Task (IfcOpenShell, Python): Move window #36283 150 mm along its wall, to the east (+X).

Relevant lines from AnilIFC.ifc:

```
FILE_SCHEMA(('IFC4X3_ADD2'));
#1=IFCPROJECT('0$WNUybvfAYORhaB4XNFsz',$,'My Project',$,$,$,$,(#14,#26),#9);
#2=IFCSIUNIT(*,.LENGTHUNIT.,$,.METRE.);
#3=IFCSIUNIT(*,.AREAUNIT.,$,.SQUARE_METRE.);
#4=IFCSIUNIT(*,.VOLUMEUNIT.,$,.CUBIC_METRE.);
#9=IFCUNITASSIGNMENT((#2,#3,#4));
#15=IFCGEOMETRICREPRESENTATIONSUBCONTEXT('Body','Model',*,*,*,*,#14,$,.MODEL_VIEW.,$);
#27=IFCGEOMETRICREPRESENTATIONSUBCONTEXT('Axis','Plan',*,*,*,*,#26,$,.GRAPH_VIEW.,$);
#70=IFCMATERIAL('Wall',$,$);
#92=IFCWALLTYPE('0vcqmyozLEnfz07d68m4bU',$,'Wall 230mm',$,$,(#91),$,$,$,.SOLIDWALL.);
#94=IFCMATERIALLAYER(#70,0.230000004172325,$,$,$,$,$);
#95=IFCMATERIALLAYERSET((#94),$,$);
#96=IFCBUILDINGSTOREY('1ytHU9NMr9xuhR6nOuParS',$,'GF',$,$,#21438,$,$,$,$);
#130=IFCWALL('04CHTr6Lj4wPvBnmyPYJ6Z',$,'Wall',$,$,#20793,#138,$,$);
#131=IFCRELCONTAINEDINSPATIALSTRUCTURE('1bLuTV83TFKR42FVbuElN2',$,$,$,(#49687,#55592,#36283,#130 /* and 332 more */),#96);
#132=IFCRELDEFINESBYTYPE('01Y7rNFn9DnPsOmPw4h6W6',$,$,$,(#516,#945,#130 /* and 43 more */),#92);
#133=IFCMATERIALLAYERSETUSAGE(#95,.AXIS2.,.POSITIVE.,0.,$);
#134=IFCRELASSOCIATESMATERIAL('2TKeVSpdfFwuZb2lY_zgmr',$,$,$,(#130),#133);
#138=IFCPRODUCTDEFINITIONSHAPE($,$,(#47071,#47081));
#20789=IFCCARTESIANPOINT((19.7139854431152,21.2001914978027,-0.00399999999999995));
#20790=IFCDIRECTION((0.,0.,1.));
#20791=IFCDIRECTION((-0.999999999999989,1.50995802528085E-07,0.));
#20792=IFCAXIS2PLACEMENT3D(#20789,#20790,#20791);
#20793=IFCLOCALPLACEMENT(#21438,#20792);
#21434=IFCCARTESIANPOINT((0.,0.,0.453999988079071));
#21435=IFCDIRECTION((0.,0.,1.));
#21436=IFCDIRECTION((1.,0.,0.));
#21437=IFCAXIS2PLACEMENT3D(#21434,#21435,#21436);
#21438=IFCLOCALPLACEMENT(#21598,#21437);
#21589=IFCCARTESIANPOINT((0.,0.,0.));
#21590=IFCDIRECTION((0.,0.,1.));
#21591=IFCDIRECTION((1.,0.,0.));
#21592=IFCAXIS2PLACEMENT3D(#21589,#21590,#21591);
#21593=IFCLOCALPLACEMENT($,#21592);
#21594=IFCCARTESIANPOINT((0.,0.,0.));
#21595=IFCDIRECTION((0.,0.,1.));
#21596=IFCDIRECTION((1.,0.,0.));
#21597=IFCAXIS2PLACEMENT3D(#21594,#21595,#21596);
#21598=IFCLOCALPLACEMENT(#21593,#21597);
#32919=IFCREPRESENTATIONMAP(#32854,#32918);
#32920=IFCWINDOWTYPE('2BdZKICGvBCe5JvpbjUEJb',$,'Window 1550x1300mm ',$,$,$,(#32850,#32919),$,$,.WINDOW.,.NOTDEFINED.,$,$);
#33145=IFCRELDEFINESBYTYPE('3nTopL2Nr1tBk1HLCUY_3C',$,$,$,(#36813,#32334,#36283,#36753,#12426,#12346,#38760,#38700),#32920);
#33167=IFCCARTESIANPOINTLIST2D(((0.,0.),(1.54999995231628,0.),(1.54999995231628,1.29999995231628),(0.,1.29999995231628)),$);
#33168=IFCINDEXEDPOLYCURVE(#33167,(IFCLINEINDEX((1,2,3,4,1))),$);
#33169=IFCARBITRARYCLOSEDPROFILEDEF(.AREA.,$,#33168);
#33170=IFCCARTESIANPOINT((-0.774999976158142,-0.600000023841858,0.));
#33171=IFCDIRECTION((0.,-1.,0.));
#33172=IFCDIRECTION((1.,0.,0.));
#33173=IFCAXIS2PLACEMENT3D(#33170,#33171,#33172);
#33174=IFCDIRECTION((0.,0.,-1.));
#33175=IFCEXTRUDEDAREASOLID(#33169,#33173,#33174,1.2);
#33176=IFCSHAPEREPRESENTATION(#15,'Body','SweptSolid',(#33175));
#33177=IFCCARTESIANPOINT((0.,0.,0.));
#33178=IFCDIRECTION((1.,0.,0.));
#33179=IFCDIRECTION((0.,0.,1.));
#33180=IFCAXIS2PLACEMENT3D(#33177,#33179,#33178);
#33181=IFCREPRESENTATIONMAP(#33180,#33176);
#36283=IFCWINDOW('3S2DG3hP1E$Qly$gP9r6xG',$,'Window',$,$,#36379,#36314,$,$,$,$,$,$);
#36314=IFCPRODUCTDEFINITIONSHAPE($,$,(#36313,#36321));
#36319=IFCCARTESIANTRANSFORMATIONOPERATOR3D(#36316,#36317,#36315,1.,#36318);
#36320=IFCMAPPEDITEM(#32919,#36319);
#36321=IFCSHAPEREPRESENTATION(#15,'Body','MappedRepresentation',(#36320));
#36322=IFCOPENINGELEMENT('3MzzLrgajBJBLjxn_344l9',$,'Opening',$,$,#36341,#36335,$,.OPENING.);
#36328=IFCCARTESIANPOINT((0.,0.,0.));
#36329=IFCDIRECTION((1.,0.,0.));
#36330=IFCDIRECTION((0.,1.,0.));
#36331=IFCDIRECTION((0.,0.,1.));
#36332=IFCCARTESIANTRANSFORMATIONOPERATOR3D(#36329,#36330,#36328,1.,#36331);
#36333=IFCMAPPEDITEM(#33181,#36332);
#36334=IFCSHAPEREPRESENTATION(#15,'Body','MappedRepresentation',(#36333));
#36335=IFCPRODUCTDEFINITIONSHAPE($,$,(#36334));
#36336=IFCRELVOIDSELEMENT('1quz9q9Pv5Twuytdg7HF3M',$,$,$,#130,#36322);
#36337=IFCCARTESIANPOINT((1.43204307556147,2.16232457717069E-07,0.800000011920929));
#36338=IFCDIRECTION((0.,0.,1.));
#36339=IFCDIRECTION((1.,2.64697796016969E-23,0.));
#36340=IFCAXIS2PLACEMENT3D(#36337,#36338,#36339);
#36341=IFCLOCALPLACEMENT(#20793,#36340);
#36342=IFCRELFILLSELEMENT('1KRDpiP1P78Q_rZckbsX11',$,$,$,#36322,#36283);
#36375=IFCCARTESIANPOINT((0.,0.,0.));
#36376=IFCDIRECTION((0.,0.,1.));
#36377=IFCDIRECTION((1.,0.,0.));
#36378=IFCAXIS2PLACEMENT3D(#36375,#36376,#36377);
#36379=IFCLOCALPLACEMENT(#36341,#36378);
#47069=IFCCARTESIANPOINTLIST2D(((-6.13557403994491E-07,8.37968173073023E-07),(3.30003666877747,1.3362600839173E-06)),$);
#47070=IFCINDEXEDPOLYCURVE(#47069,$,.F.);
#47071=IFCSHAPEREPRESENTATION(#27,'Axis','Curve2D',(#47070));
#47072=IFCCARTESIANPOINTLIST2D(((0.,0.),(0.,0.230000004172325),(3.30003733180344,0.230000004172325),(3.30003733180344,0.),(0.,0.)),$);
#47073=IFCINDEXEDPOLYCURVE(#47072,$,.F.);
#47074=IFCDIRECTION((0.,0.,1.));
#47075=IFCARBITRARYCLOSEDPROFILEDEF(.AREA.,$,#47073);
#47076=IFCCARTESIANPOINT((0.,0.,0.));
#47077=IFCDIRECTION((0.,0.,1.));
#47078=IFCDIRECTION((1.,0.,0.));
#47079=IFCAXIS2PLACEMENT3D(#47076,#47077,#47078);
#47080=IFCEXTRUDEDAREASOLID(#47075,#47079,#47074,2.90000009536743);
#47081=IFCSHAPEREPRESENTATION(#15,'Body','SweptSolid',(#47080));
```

```python
import ifcopenshell
import ifcopenshell.api.geometry
import ifcopenshell.util.placement
import ifcopenshell.util.unit

model = ifcopenshell.open("AnilIFC.ifc")
unit_scale = ifcopenshell.util.unit.calculate_unit_scale(model)

window = model.by_guid("3S2DG3hP1E$Qly$gP9r6xG")
opening = window.FillsVoids[0].RelatingOpeningElement
wall = opening.VoidsElements[0].RelatingBuildingElement

wall_matrix = ifcopenshell.util.placement.get_local_placement(wall.ObjectPlacement)
shift = wall_matrix[:3, 0] * -0.15 / unit_scale
before = ifcopenshell.util.placement.get_local_placement(window.ObjectPlacement)[:3, 3].copy()

# The window is placed relative to its opening, so it follows when the opening moves.
matrix = ifcopenshell.util.placement.get_local_placement(opening.ObjectPlacement)
matrix[:3, 3] += shift
ifcopenshell.api.geometry.edit_object_placement(
    model, product=opening, matrix=matrix, is_si=False, should_transform_children=True
)

after = ifcopenshell.util.placement.get_local_placement(window.ObjectPlacement)[:3, 3]
print("window moved by", (after - before).round(3) + 0.0)

model.write("AnilIFC_rev.ifc")
```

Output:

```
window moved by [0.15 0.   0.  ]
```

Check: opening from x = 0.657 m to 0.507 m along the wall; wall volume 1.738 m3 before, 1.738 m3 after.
